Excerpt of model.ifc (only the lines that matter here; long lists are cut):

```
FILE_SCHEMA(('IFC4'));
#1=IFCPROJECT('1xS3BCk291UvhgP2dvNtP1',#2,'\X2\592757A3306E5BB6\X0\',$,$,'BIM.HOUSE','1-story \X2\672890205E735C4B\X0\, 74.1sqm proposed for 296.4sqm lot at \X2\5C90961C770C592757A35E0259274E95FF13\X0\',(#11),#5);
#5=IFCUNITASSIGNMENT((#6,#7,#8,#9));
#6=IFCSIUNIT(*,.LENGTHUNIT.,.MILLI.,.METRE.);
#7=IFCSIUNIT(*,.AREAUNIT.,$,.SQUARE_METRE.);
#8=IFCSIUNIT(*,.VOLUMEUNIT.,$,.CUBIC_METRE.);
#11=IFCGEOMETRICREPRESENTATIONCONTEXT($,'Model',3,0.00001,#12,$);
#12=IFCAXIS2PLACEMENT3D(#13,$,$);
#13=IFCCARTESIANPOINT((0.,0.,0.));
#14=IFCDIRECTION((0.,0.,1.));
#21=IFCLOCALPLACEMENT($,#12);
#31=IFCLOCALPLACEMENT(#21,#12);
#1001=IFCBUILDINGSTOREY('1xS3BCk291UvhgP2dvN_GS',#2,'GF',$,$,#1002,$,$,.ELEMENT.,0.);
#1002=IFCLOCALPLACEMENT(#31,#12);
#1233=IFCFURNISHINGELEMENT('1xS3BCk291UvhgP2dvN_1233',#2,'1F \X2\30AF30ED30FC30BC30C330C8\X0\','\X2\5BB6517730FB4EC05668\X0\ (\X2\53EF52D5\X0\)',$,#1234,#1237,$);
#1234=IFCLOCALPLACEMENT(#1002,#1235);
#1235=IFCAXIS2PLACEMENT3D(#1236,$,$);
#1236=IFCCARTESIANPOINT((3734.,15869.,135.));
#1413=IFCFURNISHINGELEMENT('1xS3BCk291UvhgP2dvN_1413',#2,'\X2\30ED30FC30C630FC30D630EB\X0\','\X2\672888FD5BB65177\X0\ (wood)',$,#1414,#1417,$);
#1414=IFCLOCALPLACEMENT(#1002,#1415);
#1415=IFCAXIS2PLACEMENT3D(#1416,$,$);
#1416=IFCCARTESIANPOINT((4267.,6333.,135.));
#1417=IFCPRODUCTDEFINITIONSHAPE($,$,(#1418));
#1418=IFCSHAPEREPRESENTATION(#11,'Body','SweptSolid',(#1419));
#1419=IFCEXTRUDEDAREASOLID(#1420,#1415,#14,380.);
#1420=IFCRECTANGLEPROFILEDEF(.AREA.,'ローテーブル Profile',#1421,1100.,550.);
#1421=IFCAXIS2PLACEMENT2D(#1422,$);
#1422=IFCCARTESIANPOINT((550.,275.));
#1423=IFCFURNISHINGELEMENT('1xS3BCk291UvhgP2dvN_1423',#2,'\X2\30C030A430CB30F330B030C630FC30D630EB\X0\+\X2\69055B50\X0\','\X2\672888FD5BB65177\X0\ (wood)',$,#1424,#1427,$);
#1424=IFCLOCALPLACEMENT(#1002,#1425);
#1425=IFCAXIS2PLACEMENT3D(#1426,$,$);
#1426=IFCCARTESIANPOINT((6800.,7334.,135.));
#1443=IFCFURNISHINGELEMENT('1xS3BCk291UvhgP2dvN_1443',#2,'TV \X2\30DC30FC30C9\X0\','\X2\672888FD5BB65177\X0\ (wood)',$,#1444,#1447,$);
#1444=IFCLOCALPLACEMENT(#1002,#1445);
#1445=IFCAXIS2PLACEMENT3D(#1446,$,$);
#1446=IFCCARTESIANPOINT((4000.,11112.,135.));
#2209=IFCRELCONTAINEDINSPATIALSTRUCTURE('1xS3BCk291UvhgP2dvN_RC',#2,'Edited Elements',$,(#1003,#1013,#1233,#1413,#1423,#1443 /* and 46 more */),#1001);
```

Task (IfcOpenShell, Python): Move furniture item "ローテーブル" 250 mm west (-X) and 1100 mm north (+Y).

```python
import ifcopenshell
import ifcopenshell.api.geometry
import ifcopenshell.util.placement
import ifcopenshell.util.unit

model = ifcopenshell.open("model.ifc")
unit_scale = ifcopenshell.util.unit.calculate_unit_scale(model)

item = model.by_id(1413)
matrix = ifcopenshell.util.placement.get_local_placement(item.ObjectPlacement)
matrix[0, 3] -= 0.25 / unit_scale
matrix[1, 3] += 1.1 / unit_scale
ifcopenshell.api.geometry.edit_object_placement(model, product=item, matrix=matrix, is_si=False)

print(ifcopenshell.util.placement.get_local_placement(item.ObjectPlacement).round(3) + 0.0)

model.write("model-out.ifc")
```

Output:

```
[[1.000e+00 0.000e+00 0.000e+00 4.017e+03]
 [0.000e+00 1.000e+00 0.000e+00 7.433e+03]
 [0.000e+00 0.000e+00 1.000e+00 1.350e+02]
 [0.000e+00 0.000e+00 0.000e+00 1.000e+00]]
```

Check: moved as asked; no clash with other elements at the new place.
